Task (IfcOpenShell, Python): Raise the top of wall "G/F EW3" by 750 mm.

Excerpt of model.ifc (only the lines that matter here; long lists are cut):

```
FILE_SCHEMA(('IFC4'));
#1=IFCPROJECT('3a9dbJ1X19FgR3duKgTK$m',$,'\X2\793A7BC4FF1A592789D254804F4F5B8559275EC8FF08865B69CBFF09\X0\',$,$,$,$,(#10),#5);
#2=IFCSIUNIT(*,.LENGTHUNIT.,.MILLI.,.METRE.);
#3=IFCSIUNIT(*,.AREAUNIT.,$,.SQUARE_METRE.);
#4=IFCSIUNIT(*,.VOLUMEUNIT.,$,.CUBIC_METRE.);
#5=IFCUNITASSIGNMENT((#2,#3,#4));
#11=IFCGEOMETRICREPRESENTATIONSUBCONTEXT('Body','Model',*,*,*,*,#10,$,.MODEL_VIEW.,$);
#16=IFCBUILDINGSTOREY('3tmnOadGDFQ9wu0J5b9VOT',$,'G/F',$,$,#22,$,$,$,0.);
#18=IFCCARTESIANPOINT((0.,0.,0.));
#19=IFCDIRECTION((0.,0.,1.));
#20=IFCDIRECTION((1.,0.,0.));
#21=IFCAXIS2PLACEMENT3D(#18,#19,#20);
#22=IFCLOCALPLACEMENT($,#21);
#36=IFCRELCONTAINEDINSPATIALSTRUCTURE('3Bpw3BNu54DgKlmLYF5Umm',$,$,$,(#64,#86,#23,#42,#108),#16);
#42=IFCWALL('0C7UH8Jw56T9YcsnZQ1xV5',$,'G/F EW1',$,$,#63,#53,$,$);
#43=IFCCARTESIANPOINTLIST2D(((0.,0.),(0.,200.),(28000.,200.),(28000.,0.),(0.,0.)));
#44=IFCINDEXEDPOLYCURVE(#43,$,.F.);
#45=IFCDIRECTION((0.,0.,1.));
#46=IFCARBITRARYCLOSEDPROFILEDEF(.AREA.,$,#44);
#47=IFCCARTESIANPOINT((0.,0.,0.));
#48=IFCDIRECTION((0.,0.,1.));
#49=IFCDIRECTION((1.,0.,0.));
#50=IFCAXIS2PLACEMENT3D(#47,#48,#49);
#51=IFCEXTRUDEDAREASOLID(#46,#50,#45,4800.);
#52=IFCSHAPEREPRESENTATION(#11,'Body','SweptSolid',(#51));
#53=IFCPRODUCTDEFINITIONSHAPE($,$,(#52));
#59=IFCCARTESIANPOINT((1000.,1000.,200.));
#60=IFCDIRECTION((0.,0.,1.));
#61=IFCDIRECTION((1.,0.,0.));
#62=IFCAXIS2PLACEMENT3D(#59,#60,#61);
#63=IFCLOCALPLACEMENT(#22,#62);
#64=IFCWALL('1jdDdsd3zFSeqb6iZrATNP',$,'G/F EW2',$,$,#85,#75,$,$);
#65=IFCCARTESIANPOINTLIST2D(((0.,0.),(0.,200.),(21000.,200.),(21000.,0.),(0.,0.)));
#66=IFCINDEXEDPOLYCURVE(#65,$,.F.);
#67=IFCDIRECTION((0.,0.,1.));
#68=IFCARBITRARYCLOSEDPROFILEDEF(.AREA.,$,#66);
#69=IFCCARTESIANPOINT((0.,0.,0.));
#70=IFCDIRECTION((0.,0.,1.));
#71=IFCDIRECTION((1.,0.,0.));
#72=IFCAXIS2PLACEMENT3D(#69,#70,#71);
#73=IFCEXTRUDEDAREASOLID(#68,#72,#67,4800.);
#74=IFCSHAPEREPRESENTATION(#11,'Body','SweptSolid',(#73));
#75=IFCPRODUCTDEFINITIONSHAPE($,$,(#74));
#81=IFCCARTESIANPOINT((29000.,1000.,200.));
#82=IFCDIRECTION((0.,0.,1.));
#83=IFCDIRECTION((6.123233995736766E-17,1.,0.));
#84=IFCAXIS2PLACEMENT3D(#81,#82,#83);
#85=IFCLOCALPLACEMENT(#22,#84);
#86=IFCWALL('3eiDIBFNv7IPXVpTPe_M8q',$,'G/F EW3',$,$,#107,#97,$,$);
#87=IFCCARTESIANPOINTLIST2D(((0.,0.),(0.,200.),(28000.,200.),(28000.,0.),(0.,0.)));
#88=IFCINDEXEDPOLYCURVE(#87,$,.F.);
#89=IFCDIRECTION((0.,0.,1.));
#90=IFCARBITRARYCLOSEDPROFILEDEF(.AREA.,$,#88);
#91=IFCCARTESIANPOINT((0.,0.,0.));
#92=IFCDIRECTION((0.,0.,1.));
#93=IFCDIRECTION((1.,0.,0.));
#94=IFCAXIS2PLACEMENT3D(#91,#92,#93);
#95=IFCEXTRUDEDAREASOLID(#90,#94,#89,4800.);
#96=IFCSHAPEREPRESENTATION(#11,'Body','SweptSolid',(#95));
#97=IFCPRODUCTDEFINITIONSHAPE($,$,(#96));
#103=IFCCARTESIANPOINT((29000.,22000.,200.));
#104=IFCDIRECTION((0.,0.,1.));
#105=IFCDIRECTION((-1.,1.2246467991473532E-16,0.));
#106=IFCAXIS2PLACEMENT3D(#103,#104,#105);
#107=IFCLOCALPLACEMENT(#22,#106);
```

```python
import ifcopenshell
import ifcopenshell.geom
import ifcopenshell.util.representation
import ifcopenshell.util.shape

model = ifcopenshell.open("model.ifc")
settings = ifcopenshell.geom.settings()


def volume(element):
    """Net volume in cubic metres, openings subtracted."""
    shape = ifcopenshell.geom.create_shape(settings, element)
    return ifcopenshell.util.shape.get_volume(shape.geometry)


wall = model.by_id(86)
before = volume(wall)

body = ifcopenshell.util.representation.get_representation(wall, "Model", "Body")
solid = body.Items[0]
old_height = solid.Depth
solid.Depth += 750.0
after = volume(wall)

print(f"height {old_height:g} -> {solid.Depth:g}, volume {before:.3f} -> {after:.3f} m3")

model.write("model_v2.ifc")
```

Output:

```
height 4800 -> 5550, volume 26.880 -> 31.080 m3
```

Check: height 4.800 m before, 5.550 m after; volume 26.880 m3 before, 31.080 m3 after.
